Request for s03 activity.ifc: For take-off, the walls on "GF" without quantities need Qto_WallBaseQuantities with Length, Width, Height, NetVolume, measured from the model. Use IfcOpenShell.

First a look at what the model holds.

```python
import ifcopenshell
import ifcopenshell.util.element
import ifcopenshell.util.unit

model = ifcopenshell.open("s03 activity.ifc")
print(model.schema)
for unit_type in ("LENGTHUNIT", "AREAUNIT", "VOLUMEUNIT"):
    print(unit_type, ifcopenshell.util.unit.calculate_unit_scale(model, unit_type))
storey = next(s for s in model.by_type("IfcBuildingStorey") if s.Name == "GF")
walls = [e for e in ifcopenshell.util.element.get_decomposition(storey) if e.is_a("IfcWall")]
for e in sorted(walls, key=lambda e: e.id()):
    print(e.id(), e.is_a(), e.Name, list(ifcopenshell.util.element.get_psets(e, qtos_only=True)), sep=" | ")
```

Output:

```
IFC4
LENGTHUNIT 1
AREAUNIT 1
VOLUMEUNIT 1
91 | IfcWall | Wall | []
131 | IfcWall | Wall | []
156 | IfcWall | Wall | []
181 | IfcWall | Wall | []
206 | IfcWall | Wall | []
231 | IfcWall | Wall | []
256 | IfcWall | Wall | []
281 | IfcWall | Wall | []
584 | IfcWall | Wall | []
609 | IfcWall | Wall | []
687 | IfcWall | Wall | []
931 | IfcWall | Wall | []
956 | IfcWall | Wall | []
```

```python
import ifcopenshell
import ifcopenshell.api.pset
import ifcopenshell.geom
import ifcopenshell.util.element
import ifcopenshell.util.shape
import ifcopenshell.util.unit

model = ifcopenshell.open("s03 activity.ifc")
unit_scale = ifcopenshell.util.unit.calculate_unit_scale(model)
volume_scale = ifcopenshell.util.unit.calculate_unit_scale(model, "VOLUMEUNIT")
settings = ifcopenshell.geom.settings()

storey = next(s for s in model.by_type("IfcBuildingStorey") if s.Name == "GF")
walls = [e for e in ifcopenshell.util.element.get_decomposition(storey) if e.is_a("IfcWall")]

for e in sorted(walls, key=lambda e: e.id()):
    if ifcopenshell.util.element.get_psets(e, qtos_only=True, should_inherit=False):
        continue
    # Geometry comes back in metres, in the element's own axes.
    shape = ifcopenshell.geom.create_shape(settings, e)
    values = {
        "Length": ifcopenshell.util.shape.get_x(shape.geometry) / unit_scale,
        "Width": ifcopenshell.util.shape.get_y(shape.geometry) / unit_scale,
        "Height": ifcopenshell.util.shape.get_z(shape.geometry) / unit_scale,
        "NetVolume": ifcopenshell.util.shape.get_volume(shape.geometry) / volume_scale,
    }
    qto = ifcopenshell.api.pset.add_qto(model, product=e, name="Qto_WallBaseQuantities")
    ifcopenshell.api.pset.edit_qto(model, qto=qto, properties=values)
    print(e.id(), {k: round(v, 3) for k, v in values.items()})

model.write("s03 activity-out.ifc")
```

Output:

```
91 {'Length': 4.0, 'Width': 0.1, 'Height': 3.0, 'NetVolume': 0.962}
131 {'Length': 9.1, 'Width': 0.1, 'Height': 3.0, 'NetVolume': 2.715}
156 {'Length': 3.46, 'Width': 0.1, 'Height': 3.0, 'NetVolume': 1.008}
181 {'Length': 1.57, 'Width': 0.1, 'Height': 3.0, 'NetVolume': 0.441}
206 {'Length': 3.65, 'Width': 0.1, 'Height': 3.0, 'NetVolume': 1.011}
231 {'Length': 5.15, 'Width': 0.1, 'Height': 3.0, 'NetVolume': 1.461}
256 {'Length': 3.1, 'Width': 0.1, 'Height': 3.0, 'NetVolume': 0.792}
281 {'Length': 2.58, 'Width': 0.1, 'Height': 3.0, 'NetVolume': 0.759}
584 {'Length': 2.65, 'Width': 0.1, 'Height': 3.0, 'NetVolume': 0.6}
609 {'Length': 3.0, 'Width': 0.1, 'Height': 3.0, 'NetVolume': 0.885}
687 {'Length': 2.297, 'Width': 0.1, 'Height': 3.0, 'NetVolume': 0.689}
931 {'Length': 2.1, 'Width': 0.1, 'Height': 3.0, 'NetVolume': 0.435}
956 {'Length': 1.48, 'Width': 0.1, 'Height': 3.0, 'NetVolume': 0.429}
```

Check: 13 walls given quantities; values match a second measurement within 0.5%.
